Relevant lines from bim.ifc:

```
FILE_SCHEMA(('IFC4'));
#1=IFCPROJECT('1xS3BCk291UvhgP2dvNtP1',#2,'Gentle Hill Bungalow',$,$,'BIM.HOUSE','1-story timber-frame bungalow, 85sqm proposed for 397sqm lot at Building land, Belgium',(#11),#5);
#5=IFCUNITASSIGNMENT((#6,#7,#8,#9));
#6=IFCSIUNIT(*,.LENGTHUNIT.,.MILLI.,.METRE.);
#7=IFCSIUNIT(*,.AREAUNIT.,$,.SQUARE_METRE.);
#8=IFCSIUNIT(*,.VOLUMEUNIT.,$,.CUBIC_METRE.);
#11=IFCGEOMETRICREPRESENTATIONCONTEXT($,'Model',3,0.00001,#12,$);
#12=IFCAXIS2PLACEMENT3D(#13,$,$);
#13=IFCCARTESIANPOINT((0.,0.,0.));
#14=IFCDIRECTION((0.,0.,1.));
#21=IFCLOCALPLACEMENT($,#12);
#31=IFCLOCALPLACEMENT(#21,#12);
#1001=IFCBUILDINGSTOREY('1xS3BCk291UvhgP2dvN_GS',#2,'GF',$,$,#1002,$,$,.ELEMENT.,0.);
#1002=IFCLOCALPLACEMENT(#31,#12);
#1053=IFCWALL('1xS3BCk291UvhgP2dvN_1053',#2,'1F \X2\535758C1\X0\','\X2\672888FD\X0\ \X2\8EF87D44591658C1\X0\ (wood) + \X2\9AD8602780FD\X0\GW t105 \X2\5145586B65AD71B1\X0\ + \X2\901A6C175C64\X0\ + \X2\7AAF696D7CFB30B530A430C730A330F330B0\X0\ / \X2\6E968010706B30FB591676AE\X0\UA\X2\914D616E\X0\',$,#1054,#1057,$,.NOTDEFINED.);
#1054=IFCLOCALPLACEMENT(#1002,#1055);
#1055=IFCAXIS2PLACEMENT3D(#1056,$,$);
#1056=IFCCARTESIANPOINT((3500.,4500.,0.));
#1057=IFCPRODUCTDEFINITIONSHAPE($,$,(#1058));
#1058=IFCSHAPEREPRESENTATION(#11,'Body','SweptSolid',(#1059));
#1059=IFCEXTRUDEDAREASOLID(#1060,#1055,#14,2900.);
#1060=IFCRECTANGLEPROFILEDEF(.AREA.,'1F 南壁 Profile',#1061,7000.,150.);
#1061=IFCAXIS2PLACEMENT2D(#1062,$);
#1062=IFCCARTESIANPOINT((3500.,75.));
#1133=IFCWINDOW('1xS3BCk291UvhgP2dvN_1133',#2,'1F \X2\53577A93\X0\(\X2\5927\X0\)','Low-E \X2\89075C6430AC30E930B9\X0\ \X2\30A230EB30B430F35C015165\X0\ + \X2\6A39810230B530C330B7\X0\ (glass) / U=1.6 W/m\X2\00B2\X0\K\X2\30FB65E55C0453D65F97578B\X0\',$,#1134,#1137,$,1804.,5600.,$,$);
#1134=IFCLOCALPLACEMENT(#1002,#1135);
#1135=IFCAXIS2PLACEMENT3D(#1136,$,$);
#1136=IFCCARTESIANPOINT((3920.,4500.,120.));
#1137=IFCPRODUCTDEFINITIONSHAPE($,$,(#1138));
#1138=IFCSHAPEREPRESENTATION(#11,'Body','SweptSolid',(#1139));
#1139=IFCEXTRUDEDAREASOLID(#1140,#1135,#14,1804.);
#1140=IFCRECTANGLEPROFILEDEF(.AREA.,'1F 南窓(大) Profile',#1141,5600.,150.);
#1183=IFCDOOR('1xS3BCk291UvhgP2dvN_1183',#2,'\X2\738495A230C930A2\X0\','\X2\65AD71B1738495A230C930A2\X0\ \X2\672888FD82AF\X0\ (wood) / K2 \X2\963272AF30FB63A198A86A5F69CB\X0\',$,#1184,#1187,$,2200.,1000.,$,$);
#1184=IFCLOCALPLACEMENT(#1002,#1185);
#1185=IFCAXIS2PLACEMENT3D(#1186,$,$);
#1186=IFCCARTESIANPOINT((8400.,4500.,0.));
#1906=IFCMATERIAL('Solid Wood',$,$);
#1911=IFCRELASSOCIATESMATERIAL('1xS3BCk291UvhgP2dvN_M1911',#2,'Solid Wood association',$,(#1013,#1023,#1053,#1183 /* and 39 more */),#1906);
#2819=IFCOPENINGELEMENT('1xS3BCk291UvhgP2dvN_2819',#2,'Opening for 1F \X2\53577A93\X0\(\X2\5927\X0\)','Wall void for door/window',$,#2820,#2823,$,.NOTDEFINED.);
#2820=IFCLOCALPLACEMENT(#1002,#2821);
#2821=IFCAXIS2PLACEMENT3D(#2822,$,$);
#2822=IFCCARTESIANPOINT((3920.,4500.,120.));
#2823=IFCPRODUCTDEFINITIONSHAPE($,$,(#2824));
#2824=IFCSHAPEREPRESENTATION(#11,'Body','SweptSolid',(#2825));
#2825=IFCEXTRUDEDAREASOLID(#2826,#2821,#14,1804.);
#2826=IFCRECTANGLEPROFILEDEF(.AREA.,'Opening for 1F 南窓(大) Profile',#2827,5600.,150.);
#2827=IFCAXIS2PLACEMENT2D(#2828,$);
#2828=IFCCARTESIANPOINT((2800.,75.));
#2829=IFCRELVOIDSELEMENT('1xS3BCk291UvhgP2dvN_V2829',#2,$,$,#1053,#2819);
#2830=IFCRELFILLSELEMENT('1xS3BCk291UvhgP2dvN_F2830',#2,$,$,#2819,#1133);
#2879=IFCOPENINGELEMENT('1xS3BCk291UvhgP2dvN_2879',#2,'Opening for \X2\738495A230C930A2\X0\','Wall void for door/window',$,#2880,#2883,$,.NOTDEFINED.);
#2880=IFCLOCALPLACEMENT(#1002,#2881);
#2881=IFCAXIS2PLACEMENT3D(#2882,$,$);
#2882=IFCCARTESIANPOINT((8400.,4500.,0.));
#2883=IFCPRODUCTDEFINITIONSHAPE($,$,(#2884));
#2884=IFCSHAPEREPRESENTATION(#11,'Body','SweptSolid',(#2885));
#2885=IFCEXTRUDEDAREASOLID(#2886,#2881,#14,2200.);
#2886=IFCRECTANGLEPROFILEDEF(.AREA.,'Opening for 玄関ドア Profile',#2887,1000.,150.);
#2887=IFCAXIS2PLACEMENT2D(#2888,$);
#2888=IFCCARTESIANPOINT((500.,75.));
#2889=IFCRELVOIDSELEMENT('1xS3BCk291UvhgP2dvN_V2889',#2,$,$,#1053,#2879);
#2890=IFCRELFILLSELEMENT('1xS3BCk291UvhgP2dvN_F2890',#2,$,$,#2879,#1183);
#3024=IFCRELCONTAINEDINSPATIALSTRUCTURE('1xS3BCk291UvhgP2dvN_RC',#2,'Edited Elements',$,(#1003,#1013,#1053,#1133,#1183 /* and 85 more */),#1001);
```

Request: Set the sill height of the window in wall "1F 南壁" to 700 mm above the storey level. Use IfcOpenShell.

```python
import numpy as np
import ifcopenshell
import ifcopenshell.api.geometry
import ifcopenshell.geom
import ifcopenshell.util.element
import ifcopenshell.util.placement
import ifcopenshell.util.shape
import ifcopenshell.util.unit

model = ifcopenshell.open("bim.ifc")
unit_scale = ifcopenshell.util.unit.calculate_unit_scale(model)

window = model.by_guid("1xS3BCk291UvhgP2dvN_1133")
opening = window.FillsVoids[0].RelatingOpeningElement
storey = ifcopenshell.util.element.get_container(window, ifc_class="IfcBuildingStorey")
level = ifcopenshell.util.placement.get_local_placement(storey.ObjectPlacement)[2, 3]

# The opening's origin need not be at the sill, so measure its lowest point.
shape = ifcopenshell.geom.create_shape(ifcopenshell.geom.settings(), opening)
bottom = ifcopenshell.util.shape.get_shape_bottom_elevation(shape, shape.geometry) / unit_scale
dz = level + 700.0 - bottom

shift = np.array([0.0, 0.0, dz])
# The window is not placed relative to its opening, so move both.
for product in (opening, window):
    matrix = ifcopenshell.util.placement.get_local_placement(product.ObjectPlacement)
    matrix[:3, 3] += shift
    ifcopenshell.api.geometry.edit_object_placement(model, product=product, matrix=matrix, is_si=False)

print(f"moved by {dz * unit_scale:+.3f} m")

model.write("bim_rev.ifc")
```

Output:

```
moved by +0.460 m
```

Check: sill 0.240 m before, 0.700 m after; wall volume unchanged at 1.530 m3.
